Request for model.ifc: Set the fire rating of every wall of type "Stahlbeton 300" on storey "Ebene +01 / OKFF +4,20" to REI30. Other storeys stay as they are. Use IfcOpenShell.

First a look at what the model holds.

```python
import ifcopenshell
import ifcopenshell.util.element

model = ifcopenshell.open("model.ifc")
print(model.schema)
storey = next(s for s in model.by_type("IfcBuildingStorey") if s.Name == "Ebene +01 / OKFF +4,20")
walls = [e for e in ifcopenshell.util.element.get_decomposition(storey) if e.is_a("IfcWall")]
seen = {}
for e in walls:
    element_type = ifcopenshell.util.element.get_type(e)
    key = (element_type.Name if element_type != e and element_type else None, ifcopenshell.util.element.get_pset(e, "Pset_WallCommon", "FireRating"))
    seen[key] = seen.get(key, 0) + 1
for (name, value), count in sorted(seen.items(), key=str):
    print(count, "x", name, "|", value)
```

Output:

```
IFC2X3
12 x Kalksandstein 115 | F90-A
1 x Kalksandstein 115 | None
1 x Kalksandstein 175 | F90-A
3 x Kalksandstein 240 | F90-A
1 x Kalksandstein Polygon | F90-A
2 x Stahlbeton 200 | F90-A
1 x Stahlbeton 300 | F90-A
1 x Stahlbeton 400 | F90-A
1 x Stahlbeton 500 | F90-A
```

```python
import ifcopenshell
import ifcopenshell.api.pset
import ifcopenshell.util.element

model = ifcopenshell.open("model.ifc")

storey = next(s for s in model.by_type("IfcBuildingStorey") if s.Name == "Ebene +01 / OKFF +4,20")
walls = [e for e in ifcopenshell.util.element.get_decomposition(storey) if e.is_a("IfcWall")]

count = 0
for e in walls:
    element_type = ifcopenshell.util.element.get_type(e)
    if element_type in (None, e) or element_type.Name != "Stahlbeton 300":
        continue
    # add_pset returns the element's existing set when there is one.
    pset = ifcopenshell.api.pset.add_pset(model, product=e, name="Pset_WallCommon")
    ifcopenshell.api.pset.edit_pset(model, pset=pset, properties={"FireRating": "REI30"})
    count += 1

print(count, "walls updated")

model.write("model_v2.ifc")
```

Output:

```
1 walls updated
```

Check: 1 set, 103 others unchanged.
